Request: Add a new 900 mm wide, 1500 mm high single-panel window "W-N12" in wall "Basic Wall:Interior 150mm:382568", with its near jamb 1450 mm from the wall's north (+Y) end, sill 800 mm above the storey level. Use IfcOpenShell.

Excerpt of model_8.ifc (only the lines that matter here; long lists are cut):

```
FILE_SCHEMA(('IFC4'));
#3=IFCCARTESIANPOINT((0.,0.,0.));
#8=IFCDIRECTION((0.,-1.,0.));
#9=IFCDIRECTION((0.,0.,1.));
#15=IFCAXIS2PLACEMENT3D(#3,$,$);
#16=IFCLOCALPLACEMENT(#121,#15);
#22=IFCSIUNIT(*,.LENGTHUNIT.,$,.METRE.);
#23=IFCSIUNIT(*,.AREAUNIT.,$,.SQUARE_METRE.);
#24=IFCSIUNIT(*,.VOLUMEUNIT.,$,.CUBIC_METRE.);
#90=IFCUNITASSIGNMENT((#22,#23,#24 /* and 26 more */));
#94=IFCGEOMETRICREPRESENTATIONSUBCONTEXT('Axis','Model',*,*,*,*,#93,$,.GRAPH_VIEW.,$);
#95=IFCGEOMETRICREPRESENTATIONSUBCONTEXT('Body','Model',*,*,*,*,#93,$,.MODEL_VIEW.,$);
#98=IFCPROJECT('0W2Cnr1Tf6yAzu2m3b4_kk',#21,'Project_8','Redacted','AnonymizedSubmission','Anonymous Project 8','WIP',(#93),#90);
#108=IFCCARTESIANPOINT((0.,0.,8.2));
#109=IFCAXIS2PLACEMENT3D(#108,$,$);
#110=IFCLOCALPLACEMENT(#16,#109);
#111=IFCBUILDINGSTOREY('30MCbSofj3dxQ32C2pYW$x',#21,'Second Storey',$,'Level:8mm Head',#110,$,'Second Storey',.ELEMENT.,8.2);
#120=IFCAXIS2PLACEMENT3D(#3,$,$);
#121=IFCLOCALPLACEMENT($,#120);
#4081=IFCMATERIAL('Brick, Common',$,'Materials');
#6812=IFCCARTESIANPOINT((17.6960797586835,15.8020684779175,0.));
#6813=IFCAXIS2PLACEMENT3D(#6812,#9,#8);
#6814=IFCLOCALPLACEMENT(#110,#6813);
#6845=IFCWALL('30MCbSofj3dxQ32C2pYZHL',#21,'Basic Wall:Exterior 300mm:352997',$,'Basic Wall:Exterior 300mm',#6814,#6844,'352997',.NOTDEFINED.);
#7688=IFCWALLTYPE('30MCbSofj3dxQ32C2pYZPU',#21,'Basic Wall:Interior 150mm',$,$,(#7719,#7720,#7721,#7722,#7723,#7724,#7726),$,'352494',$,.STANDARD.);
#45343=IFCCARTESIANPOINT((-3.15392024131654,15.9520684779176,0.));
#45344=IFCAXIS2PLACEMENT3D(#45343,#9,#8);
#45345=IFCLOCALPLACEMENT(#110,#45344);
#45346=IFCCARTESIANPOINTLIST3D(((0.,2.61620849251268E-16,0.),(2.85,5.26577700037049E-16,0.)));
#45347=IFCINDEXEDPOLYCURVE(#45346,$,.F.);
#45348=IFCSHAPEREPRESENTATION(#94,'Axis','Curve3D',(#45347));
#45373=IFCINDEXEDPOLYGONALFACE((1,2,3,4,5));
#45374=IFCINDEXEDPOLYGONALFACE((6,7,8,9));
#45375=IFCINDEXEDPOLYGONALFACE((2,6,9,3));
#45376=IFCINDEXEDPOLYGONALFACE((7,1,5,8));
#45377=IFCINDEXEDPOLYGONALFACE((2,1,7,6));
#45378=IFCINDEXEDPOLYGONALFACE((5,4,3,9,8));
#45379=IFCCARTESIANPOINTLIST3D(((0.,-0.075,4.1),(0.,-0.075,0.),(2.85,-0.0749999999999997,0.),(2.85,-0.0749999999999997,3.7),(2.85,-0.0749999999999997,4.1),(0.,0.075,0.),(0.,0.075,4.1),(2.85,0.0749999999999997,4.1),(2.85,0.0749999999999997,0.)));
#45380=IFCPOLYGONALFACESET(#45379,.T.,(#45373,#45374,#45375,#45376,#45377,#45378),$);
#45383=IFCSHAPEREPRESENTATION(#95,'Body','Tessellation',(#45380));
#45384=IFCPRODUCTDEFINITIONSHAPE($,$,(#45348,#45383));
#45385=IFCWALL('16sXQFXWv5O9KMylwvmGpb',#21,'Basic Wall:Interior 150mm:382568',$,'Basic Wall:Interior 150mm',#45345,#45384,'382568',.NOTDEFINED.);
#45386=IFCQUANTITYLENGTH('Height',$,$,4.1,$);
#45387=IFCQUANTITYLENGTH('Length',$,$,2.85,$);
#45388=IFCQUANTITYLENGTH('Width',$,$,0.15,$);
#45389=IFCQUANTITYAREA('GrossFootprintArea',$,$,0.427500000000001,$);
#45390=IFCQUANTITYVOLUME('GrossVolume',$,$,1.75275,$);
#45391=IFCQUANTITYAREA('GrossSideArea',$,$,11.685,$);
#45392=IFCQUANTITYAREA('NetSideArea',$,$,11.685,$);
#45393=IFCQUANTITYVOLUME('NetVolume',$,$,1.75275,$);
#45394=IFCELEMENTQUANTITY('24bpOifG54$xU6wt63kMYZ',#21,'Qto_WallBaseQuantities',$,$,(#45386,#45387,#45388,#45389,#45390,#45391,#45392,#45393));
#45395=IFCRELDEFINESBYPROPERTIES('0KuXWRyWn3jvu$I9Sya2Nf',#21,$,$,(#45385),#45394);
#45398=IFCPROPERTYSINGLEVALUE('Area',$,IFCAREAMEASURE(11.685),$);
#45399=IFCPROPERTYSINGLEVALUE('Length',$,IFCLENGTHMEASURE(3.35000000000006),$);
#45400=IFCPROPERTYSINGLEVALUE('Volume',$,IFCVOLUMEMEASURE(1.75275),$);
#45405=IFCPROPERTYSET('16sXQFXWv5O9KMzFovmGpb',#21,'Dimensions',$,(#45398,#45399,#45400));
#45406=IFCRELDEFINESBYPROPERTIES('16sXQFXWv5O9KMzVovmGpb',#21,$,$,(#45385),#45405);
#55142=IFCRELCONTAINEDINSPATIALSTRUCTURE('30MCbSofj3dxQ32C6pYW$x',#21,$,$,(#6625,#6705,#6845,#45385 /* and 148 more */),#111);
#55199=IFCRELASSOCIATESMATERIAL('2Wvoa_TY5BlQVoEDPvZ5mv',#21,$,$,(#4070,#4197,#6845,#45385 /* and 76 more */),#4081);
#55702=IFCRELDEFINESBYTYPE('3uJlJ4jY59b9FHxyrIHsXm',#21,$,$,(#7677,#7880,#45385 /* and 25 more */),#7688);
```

```python
import numpy as np
import ifcopenshell
import ifcopenshell.api.feature
import ifcopenshell.api.geometry
import ifcopenshell.api.pset
import ifcopenshell.api.root
import ifcopenshell.api.spatial
import ifcopenshell.geom
import ifcopenshell.util.element
import ifcopenshell.util.placement
import ifcopenshell.util.representation
import ifcopenshell.util.shape
import ifcopenshell.util.unit

model = ifcopenshell.open("model_8.ifc")
unit_scale = ifcopenshell.util.unit.calculate_unit_scale(model)
area_scale = ifcopenshell.util.unit.calculate_unit_scale(model, "AREAUNIT")
volume_scale = ifcopenshell.util.unit.calculate_unit_scale(model, "VOLUMEUNIT")
settings = ifcopenshell.geom.settings()


def volume(element):
    """Net volume in cubic metres, openings subtracted."""
    shape = ifcopenshell.geom.create_shape(settings, element)
    return ifcopenshell.util.shape.get_volume(shape.geometry)


wall = model.by_guid("16sXQFXWv5O9KMylwvmGpb")
storey = ifcopenshell.util.element.get_container(wall, ifc_class="IfcBuildingStorey")
context = ifcopenshell.util.representation.get_context(model, "Model", "Body", "MODEL_VIEW")
before = volume(wall)

width, height, from_end, sill = 0.9, 1.5, 1.45, 0.8  # metres

# The wall runs along its own X axis, and the end named is its -X end.
wall_shape = ifcopenshell.geom.create_shape(settings, wall)
x, y, z = ifcopenshell.util.shape.get_vertices(wall_shape.geometry).T
start = x.min() + from_end
face, thickness = float(y.min()), float(y.max() - y.min())
wall_matrix = ifcopenshell.util.placement.get_local_placement(wall.ObjectPlacement)
level = ifcopenshell.util.placement.get_local_placement(storey.ObjectPlacement)[2, 3]


def in_wall(x, y):
    """Placement at x, y metres in the wall's axes, at sill height."""
    matrix = wall_matrix.copy()
    matrix[:, 3] = wall_matrix @ np.array([x / unit_scale, y / unit_scale, 0.0, 1.0])
    matrix[2, 3] = level + sill / unit_scale
    return matrix


# Opening: a box that overshoots both wall faces by 50 mm.
opening = ifcopenshell.api.root.create_entity(model, ifc_class="IfcOpeningElement", predefined_type="OPENING")
box = ifcopenshell.api.geometry.add_wall_representation(
    model, context=context, length=width, height=height, thickness=thickness + 0.1
)
ifcopenshell.api.geometry.assign_representation(model, product=opening, representation=box)
ifcopenshell.api.geometry.edit_object_placement(model, product=opening, matrix=in_wall(start, face - 0.05), is_si=False)
ifcopenshell.api.feature.add_feature(model, feature=opening, element=wall)

window = ifcopenshell.api.root.create_entity(model, ifc_class="IfcWindow", name="W-N12", predefined_type="WINDOW")
window.OverallWidth, window.OverallHeight = width / unit_scale, height / unit_scale
window.PartitioningType = "SINGLE_PANEL"
body = ifcopenshell.api.geometry.add_window_representation(
    model,
    context=context,
    overall_width=window.OverallWidth,
    overall_height=window.OverallHeight,
    partition_type="SINGLE_PANEL",
)
ifcopenshell.api.geometry.assign_representation(model, product=window, representation=body)
ifcopenshell.api.spatial.assign_container(model, products=[window], relating_structure=storey)
ifcopenshell.api.feature.add_filling(model, opening=opening, element=window)

# Centre the window in the wall's thickness.
ifcopenshell.api.geometry.edit_object_placement(model, product=window, matrix=in_wall(start, face), is_si=False)
window_shape = ifcopenshell.geom.create_shape(settings, window)
depth = ifcopenshell.util.shape.get_vertices(window_shape.geometry)[:, 1]
offset = face + thickness / 2 - (depth.min() + depth.max()) / 2
ifcopenshell.api.geometry.edit_object_placement(model, product=window, matrix=in_wall(start, offset), is_si=False)

after = volume(wall)

# Update the wall's stored quantities.
qto = model.by_id(ifcopenshell.util.element.get_pset(wall, "Qto_WallBaseQuantities", should_inherit=False)["id"])
ifcopenshell.api.pset.edit_qto(model, qto=qto, properties={
    "NetSideArea": after / thickness / area_scale,
    "NetVolume": after / volume_scale,
})
pset = model.by_id(ifcopenshell.util.element.get_pset(wall, "Dimensions", should_inherit=False)["id"])
ifcopenshell.api.pset.edit_pset(model, pset=pset, properties={
    "Area": model.create_entity("IfcAreaMeasure", after / thickness / area_scale),
    "Volume": model.create_entity("IfcVolumeMeasure", after / volume_scale),
})

print(f"wall volume {before:.3f} -> {after:.3f} m3")

model.write("model_8_edited.ifc")
```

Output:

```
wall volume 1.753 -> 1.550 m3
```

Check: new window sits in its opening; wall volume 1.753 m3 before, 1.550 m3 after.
